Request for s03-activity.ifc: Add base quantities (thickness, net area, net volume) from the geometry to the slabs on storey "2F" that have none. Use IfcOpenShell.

First a look at what the model holds.

```python
import ifcopenshell
import ifcopenshell.util.element
import ifcopenshell.util.unit

model = ifcopenshell.open("s03-activity.ifc")
print(model.schema)
for unit_type in ("LENGTHUNIT", "AREAUNIT", "VOLUMEUNIT"):
    print(unit_type, ifcopenshell.util.unit.calculate_unit_scale(model, unit_type))
storey = next(s for s in model.by_type("IfcBuildingStorey") if s.Name == "2F")
slabs = [e for e in ifcopenshell.util.element.get_decomposition(storey) if e.is_a("IfcSlab")]
for e in sorted(slabs, key=lambda e: e.id()):
    print(e.id(), e.is_a(), e.Name, list(ifcopenshell.util.element.get_psets(e, qtos_only=True)), sep=" | ")
```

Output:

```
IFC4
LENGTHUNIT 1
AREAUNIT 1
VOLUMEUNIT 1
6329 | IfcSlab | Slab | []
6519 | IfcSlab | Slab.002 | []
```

```python
import ifcopenshell
import ifcopenshell.api.pset
import ifcopenshell.geom
import ifcopenshell.util.element
import ifcopenshell.util.shape
import ifcopenshell.util.unit

model = ifcopenshell.open("s03-activity.ifc")
unit_scale = ifcopenshell.util.unit.calculate_unit_scale(model)
area_scale = ifcopenshell.util.unit.calculate_unit_scale(model, "AREAUNIT")
volume_scale = ifcopenshell.util.unit.calculate_unit_scale(model, "VOLUMEUNIT")
settings = ifcopenshell.geom.settings()

storey = next(s for s in model.by_type("IfcBuildingStorey") if s.Name == "2F")
slabs = [e for e in ifcopenshell.util.element.get_decomposition(storey) if e.is_a("IfcSlab")]

for e in sorted(slabs, key=lambda e: e.id()):
    if ifcopenshell.util.element.get_psets(e, qtos_only=True, should_inherit=False):
        continue
    # Geometry comes back in metres, in the element's own axes.
    shape = ifcopenshell.geom.create_shape(settings, e)
    values = {
        "Width": ifcopenshell.util.shape.get_z(shape.geometry) / unit_scale,
        "NetArea": ifcopenshell.util.shape.get_footprint_area(shape.geometry) / area_scale,
        "NetVolume": ifcopenshell.util.shape.get_volume(shape.geometry) / volume_scale,
    }
    qto = ifcopenshell.api.pset.add_qto(model, product=e, name="Qto_SlabBaseQuantities")
    ifcopenshell.api.pset.edit_qto(model, qto=qto, properties=values)
    print(e.id(), {k: round(v, 3) for k, v in values.items()})

model.write("s03-activity_rev.ifc")
```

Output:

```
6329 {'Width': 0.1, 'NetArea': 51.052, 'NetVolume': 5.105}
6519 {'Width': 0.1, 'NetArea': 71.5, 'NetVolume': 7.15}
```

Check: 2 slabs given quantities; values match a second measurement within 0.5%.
